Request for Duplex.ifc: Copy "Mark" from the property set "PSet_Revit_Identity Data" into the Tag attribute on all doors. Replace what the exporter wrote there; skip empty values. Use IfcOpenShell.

First a look at what the model holds.

```python
import ifcopenshell
import ifcopenshell.util.element

model = ifcopenshell.open("Duplex.ifc")
print(model.schema)
doors = model.by_type("IfcDoor")
print(len(doors), "doors")
for e in doors[:8]:
    source = ifcopenshell.util.element.get_pset(e, "PSet_Revit_Identity Data", "Mark")
    target = e.Tag
    print(e.id(), repr(source), repr(target), sep=" | ")
```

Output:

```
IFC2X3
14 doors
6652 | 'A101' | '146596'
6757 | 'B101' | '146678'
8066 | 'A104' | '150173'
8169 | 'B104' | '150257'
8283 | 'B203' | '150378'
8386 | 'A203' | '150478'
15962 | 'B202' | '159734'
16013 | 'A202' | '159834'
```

```python
import ifcopenshell
import ifcopenshell.util.element

model = ifcopenshell.open("Duplex.ifc")

count = 0
for e in model.by_type("IfcDoor"):
    value = ifcopenshell.util.element.get_pset(e, "PSet_Revit_Identity Data", "Mark")
    current = e.Tag
    if not value or not value.strip() or current == value:
        continue
    e.Tag = value
    count += 1

print(count, "doors updated")

model.write("Duplex_updated.ifc")
```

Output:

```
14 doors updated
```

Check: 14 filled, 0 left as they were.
